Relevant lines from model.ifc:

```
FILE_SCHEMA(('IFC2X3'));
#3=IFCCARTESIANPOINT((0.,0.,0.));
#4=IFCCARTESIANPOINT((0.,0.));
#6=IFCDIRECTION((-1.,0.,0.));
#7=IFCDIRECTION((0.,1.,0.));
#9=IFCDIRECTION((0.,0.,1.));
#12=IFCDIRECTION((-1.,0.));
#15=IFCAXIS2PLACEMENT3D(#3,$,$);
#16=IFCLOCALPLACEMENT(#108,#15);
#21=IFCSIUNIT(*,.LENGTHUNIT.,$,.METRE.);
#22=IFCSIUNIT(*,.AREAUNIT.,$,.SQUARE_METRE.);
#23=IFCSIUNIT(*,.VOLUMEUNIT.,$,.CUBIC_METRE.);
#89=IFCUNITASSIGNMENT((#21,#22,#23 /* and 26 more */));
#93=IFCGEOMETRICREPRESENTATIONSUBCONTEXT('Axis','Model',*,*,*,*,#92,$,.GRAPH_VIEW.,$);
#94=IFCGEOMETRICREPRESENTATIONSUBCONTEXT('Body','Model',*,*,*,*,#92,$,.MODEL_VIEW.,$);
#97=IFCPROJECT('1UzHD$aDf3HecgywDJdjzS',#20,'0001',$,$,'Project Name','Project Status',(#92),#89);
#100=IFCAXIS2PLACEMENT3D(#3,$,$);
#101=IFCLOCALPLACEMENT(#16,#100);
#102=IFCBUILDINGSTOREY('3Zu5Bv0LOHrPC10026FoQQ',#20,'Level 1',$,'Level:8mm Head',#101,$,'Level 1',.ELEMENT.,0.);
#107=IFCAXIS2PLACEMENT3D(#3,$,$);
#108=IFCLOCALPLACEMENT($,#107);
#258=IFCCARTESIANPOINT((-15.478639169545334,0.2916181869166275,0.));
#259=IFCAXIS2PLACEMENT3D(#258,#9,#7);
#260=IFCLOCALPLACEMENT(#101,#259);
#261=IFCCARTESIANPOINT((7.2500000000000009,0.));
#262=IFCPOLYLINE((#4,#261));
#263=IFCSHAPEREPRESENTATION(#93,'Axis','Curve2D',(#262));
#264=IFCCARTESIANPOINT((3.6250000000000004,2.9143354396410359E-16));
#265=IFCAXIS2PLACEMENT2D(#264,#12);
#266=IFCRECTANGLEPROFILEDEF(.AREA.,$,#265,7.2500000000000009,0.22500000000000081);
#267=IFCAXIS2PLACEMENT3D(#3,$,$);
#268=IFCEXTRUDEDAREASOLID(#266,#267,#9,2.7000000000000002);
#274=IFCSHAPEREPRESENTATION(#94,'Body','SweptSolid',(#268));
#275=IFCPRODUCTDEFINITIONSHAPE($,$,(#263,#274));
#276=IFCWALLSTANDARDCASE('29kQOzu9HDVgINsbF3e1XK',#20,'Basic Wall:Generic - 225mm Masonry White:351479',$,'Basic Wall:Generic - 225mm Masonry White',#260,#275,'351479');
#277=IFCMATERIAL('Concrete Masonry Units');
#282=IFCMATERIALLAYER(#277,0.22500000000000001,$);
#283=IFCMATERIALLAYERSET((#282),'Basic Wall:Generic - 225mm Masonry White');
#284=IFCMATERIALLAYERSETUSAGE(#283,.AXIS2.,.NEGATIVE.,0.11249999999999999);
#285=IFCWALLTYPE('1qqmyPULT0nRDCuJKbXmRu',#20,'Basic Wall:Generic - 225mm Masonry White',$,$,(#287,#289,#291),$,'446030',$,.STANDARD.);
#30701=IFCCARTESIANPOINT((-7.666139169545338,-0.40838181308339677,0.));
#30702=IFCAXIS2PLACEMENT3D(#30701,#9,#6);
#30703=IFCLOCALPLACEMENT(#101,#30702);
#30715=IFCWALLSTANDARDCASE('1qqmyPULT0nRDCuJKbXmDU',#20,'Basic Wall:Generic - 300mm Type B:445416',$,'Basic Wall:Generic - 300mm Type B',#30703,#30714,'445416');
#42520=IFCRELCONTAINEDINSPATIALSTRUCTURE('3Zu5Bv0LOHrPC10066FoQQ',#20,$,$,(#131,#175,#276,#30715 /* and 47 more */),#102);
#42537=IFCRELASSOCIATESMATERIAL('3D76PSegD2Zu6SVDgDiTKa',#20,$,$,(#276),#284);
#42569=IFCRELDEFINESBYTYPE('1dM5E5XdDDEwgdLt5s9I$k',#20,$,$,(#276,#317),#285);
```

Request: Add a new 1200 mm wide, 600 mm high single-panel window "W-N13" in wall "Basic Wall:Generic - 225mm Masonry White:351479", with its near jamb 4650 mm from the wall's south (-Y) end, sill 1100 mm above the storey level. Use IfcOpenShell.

```python
import numpy as np
import ifcopenshell
import ifcopenshell.api.feature
import ifcopenshell.api.geometry
import ifcopenshell.api.root
import ifcopenshell.api.spatial
import ifcopenshell.api.type
import ifcopenshell.geom
import ifcopenshell.util.element
import ifcopenshell.util.placement
import ifcopenshell.util.representation
import ifcopenshell.util.shape
import ifcopenshell.util.unit

model = ifcopenshell.open("model.ifc")
unit_scale = ifcopenshell.util.unit.calculate_unit_scale(model)
settings = ifcopenshell.geom.settings()


def volume(element):
    """Net volume in cubic metres, openings subtracted."""
    shape = ifcopenshell.geom.create_shape(settings, element)
    return ifcopenshell.util.shape.get_volume(shape.geometry)


wall = model.by_guid("29kQOzu9HDVgINsbF3e1XK")
storey = ifcopenshell.util.element.get_container(wall, ifc_class="IfcBuildingStorey")
context = ifcopenshell.util.representation.get_context(model, "Model", "Body", "MODEL_VIEW")
before = volume(wall)

width, height, from_end, sill = 1.2, 0.6, 4.65, 1.1  # metres

# The wall runs along its own X axis, and the end named is its -X end.
wall_shape = ifcopenshell.geom.create_shape(settings, wall)
x, y, z = ifcopenshell.util.shape.get_vertices(wall_shape.geometry).T
start = x.min() + from_end
face, thickness = float(y.min()), float(y.max() - y.min())
wall_matrix = ifcopenshell.util.placement.get_local_placement(wall.ObjectPlacement)
level = ifcopenshell.util.placement.get_local_placement(storey.ObjectPlacement)[2, 3]


def in_wall(x, y):
    """Placement at x, y metres in the wall's axes, at sill height."""
    matrix = wall_matrix.copy()
    matrix[:, 3] = wall_matrix @ np.array([x / unit_scale, y / unit_scale, 0.0, 1.0])
    matrix[2, 3] = level + sill / unit_scale
    return matrix


# Opening: a box that overshoots both wall faces by 50 mm.
opening = ifcopenshell.api.root.create_entity(model, ifc_class="IfcOpeningElement")
box = ifcopenshell.api.geometry.add_wall_representation(
    model, context=context, length=width, height=height, thickness=thickness + 0.1
)
ifcopenshell.api.geometry.assign_representation(model, product=opening, representation=box)
ifcopenshell.api.geometry.edit_object_placement(model, product=opening, matrix=in_wall(start, face - 0.05), is_si=False)
ifcopenshell.api.feature.add_feature(model, feature=opening, element=wall)

window = ifcopenshell.api.root.create_entity(model, ifc_class="IfcWindow", name="W-N13")
window.OverallWidth, window.OverallHeight = width / unit_scale, height / unit_scale
body = ifcopenshell.api.geometry.add_window_representation(
    model,
    context=context,
    overall_width=window.OverallWidth,
    overall_height=window.OverallHeight,
    partition_type="SINGLE_PANEL",
)
ifcopenshell.api.geometry.assign_representation(model, product=window, representation=body)
ifcopenshell.api.spatial.assign_container(model, products=[window], relating_structure=storey)
fills = ifcopenshell.api.feature.add_filling(model, opening=opening, element=window)
fills.OwnerHistory = window.OwnerHistory  # required in IFC2X3

# IFC2X3 keeps the operation on the window style.
style = ifcopenshell.api.root.create_entity(model, ifc_class="IfcWindowStyle", name="W-N13")
style.OperationType, style.ConstructionType = "SINGLE_PANEL", "NOTDEFINED"
style.ParameterTakesPrecedence = style.Sizeable = False
ifcopenshell.api.type.assign_type(model, related_objects=[window], relating_type=style)

# Centre the window in the wall's thickness.
ifcopenshell.api.geometry.edit_object_placement(model, product=window, matrix=in_wall(start, face), is_si=False)
window_shape = ifcopenshell.geom.create_shape(settings, window)
depth = ifcopenshell.util.shape.get_vertices(window_shape.geometry)[:, 1]
offset = face + thickness / 2 - (depth.min() + depth.max()) / 2
ifcopenshell.api.geometry.edit_object_placement(model, product=window, matrix=in_wall(start, offset), is_si=False)

after = volume(wall)

print(f"wall volume {before:.3f} -> {after:.3f} m3")

model.write("model-out.ifc")
```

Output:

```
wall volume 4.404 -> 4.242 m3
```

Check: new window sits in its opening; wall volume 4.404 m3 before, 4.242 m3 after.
